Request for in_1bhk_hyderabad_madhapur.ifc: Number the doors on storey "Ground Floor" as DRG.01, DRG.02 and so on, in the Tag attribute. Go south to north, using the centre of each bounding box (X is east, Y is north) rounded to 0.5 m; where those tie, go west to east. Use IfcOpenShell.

First a look at what the model holds.

```python
import ifcopenshell
import ifcopenshell.util.element
import ifcopenshell.util.placement

model = ifcopenshell.open("in_1bhk_hyderabad_madhapur.ifc")
print(model.schema)
storey = next(s for s in model.by_type("IfcBuildingStorey") if s.Name == "Ground Floor")
doors = [e for e in ifcopenshell.util.element.get_decomposition(storey) if e.is_a("IfcDoor")]
for e in sorted(doors, key=lambda e: e.id()):
    origin = ifcopenshell.util.placement.get_local_placement(e.ObjectPlacement)[:3, 3]
    print(e.id(), e.Tag, e.Name, origin.round(2) + 0.0, sep=" | ")
```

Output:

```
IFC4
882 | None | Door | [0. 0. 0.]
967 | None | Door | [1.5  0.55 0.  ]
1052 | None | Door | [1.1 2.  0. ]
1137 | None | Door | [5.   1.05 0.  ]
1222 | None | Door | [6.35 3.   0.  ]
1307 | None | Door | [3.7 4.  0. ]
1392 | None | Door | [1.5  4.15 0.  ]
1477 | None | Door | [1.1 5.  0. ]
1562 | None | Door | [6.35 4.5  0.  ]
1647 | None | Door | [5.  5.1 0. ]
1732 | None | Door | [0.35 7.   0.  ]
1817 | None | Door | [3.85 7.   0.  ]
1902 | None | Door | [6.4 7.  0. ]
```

```python
import ifcopenshell
import ifcopenshell.geom
import ifcopenshell.util.element
import ifcopenshell.util.shape

model = ifcopenshell.open("in_1bhk_hyderabad_madhapur.ifc")
settings = ifcopenshell.geom.settings()
settings.set("use-world-coords", True)


def centre(element):
    shape = ifcopenshell.geom.create_shape(settings, element)
    return ifcopenshell.util.shape.get_bbox_centroid(shape.geometry)


storey = next(s for s in model.by_type("IfcBuildingStorey") if s.Name == "Ground Floor")
doors = [e for e in ifcopenshell.util.element.get_decomposition(storey) if e.is_a("IfcDoor")]

# Insertion points can sit at a corner or the storey origin, so sort by the geometry (in metres).
centres = {e: centre(e) for e in doors}
doors.sort(key=lambda e: (round(centres[e][1] / 0.5), centres[e][0]))

for i, e in enumerate(doors, start=1):
    number = f"DRG.{i:02d}"
    e.Tag = number
    print(e.id(), number)

model.write("in_1bhk_hyderabad_madhapur-out.ifc")
```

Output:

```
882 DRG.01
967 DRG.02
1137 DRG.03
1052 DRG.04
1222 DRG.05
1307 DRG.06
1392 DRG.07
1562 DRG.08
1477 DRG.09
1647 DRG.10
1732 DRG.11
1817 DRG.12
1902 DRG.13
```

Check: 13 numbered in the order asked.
